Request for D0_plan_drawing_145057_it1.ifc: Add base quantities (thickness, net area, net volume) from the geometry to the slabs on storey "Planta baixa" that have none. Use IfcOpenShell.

First a look at what the model holds.

```python
import ifcopenshell
import ifcopenshell.util.element
import ifcopenshell.util.unit

model = ifcopenshell.open("D0_plan_drawing_145057_it1.ifc")
print(model.schema)
for unit_type in ("LENGTHUNIT", "AREAUNIT", "VOLUMEUNIT"):
    print(unit_type, ifcopenshell.util.unit.calculate_unit_scale(model, unit_type))
storey = next(s for s in model.by_type("IfcBuildingStorey") if s.Name == "Planta baixa")
slabs = [e for e in ifcopenshell.util.element.get_decomposition(storey) if e.is_a("IfcSlab")]
for e in sorted(slabs, key=lambda e: e.id()):
    print(e.id(), e.is_a(), e.Name, list(ifcopenshell.util.element.get_psets(e, qtos_only=True)), sep=" | ")
```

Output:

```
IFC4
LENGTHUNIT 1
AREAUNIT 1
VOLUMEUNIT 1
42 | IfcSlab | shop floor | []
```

```python
import ifcopenshell
import ifcopenshell.api.pset
import ifcopenshell.geom
import ifcopenshell.util.element
import ifcopenshell.util.shape
import ifcopenshell.util.unit

model = ifcopenshell.open("D0_plan_drawing_145057_it1.ifc")
unit_scale = ifcopenshell.util.unit.calculate_unit_scale(model)
area_scale = ifcopenshell.util.unit.calculate_unit_scale(model, "AREAUNIT")
volume_scale = ifcopenshell.util.unit.calculate_unit_scale(model, "VOLUMEUNIT")
settings = ifcopenshell.geom.settings()

storey = next(s for s in model.by_type("IfcBuildingStorey") if s.Name == "Planta baixa")
slabs = [e for e in ifcopenshell.util.element.get_decomposition(storey) if e.is_a("IfcSlab")]

for e in sorted(slabs, key=lambda e: e.id()):
    if ifcopenshell.util.element.get_psets(e, qtos_only=True, should_inherit=False):
        continue
    # Geometry comes back in metres, in the element's own axes.
    shape = ifcopenshell.geom.create_shape(settings, e)
    values = {
        "Width": ifcopenshell.util.shape.get_z(shape.geometry) / unit_scale,
        "NetArea": ifcopenshell.util.shape.get_footprint_area(shape.geometry) / area_scale,
        "NetVolume": ifcopenshell.util.shape.get_volume(shape.geometry) / volume_scale,
    }
    qto = ifcopenshell.api.pset.add_qto(model, product=e, name="Qto_SlabBaseQuantities")
    ifcopenshell.api.pset.edit_qto(model, qto=qto, properties=values)
    print(e.id(), {k: round(v, 3) for k, v in values.items()})

model.write("D0_plan_drawing_145057_it1_v2.ifc")
```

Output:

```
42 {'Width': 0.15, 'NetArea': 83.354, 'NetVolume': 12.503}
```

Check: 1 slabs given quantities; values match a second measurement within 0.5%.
